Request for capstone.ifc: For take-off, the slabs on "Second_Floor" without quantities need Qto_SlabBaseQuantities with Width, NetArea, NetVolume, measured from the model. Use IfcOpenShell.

First a look at what the model holds.

```python
import ifcopenshell
import ifcopenshell.util.element
import ifcopenshell.util.unit

model = ifcopenshell.open("capstone.ifc")
print(model.schema)
for unit_type in ("LENGTHUNIT", "AREAUNIT", "VOLUMEUNIT"):
    print(unit_type, ifcopenshell.util.unit.calculate_unit_scale(model, unit_type))
storey = next(s for s in model.by_type("IfcBuildingStorey") if s.Name == "Second_Floor")
slabs = [e for e in ifcopenshell.util.element.get_decomposition(storey) if e.is_a("IfcSlab")]
for e in sorted(slabs, key=lambda e: e.id()):
    print(e.id(), e.is_a(), e.Name, list(ifcopenshell.util.element.get_psets(e, qtos_only=True)), sep=" | ")
```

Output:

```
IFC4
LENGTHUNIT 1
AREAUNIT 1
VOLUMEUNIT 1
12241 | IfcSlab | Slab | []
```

```python
import ifcopenshell
import ifcopenshell.api.pset
import ifcopenshell.geom
import ifcopenshell.util.element
import ifcopenshell.util.shape
import ifcopenshell.util.unit

model = ifcopenshell.open("capstone.ifc")
unit_scale = ifcopenshell.util.unit.calculate_unit_scale(model)
area_scale = ifcopenshell.util.unit.calculate_unit_scale(model, "AREAUNIT")
volume_scale = ifcopenshell.util.unit.calculate_unit_scale(model, "VOLUMEUNIT")
settings = ifcopenshell.geom.settings()

storey = next(s for s in model.by_type("IfcBuildingStorey") if s.Name == "Second_Floor")
slabs = [e for e in ifcopenshell.util.element.get_decomposition(storey) if e.is_a("IfcSlab")]

for e in sorted(slabs, key=lambda e: e.id()):
    if ifcopenshell.util.element.get_psets(e, qtos_only=True, should_inherit=False):
        continue
    # Geometry comes back in metres, in the element's own axes.
    shape = ifcopenshell.geom.create_shape(settings, e)
    values = {
        "Width": ifcopenshell.util.shape.get_z(shape.geometry) / unit_scale,
        "NetArea": ifcopenshell.util.shape.get_footprint_area(shape.geometry) / area_scale,
        "NetVolume": ifcopenshell.util.shape.get_volume(shape.geometry) / volume_scale,
    }
    qto = ifcopenshell.api.pset.add_qto(model, product=e, name="Qto_SlabBaseQuantities")
    ifcopenshell.api.pset.edit_qto(model, qto=qto, properties=values)
    print(e.id(), {k: round(v, 3) for k, v in values.items()})

model.write("capstone-out.ifc")
```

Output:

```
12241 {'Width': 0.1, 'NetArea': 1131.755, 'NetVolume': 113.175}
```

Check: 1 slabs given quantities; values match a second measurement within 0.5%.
